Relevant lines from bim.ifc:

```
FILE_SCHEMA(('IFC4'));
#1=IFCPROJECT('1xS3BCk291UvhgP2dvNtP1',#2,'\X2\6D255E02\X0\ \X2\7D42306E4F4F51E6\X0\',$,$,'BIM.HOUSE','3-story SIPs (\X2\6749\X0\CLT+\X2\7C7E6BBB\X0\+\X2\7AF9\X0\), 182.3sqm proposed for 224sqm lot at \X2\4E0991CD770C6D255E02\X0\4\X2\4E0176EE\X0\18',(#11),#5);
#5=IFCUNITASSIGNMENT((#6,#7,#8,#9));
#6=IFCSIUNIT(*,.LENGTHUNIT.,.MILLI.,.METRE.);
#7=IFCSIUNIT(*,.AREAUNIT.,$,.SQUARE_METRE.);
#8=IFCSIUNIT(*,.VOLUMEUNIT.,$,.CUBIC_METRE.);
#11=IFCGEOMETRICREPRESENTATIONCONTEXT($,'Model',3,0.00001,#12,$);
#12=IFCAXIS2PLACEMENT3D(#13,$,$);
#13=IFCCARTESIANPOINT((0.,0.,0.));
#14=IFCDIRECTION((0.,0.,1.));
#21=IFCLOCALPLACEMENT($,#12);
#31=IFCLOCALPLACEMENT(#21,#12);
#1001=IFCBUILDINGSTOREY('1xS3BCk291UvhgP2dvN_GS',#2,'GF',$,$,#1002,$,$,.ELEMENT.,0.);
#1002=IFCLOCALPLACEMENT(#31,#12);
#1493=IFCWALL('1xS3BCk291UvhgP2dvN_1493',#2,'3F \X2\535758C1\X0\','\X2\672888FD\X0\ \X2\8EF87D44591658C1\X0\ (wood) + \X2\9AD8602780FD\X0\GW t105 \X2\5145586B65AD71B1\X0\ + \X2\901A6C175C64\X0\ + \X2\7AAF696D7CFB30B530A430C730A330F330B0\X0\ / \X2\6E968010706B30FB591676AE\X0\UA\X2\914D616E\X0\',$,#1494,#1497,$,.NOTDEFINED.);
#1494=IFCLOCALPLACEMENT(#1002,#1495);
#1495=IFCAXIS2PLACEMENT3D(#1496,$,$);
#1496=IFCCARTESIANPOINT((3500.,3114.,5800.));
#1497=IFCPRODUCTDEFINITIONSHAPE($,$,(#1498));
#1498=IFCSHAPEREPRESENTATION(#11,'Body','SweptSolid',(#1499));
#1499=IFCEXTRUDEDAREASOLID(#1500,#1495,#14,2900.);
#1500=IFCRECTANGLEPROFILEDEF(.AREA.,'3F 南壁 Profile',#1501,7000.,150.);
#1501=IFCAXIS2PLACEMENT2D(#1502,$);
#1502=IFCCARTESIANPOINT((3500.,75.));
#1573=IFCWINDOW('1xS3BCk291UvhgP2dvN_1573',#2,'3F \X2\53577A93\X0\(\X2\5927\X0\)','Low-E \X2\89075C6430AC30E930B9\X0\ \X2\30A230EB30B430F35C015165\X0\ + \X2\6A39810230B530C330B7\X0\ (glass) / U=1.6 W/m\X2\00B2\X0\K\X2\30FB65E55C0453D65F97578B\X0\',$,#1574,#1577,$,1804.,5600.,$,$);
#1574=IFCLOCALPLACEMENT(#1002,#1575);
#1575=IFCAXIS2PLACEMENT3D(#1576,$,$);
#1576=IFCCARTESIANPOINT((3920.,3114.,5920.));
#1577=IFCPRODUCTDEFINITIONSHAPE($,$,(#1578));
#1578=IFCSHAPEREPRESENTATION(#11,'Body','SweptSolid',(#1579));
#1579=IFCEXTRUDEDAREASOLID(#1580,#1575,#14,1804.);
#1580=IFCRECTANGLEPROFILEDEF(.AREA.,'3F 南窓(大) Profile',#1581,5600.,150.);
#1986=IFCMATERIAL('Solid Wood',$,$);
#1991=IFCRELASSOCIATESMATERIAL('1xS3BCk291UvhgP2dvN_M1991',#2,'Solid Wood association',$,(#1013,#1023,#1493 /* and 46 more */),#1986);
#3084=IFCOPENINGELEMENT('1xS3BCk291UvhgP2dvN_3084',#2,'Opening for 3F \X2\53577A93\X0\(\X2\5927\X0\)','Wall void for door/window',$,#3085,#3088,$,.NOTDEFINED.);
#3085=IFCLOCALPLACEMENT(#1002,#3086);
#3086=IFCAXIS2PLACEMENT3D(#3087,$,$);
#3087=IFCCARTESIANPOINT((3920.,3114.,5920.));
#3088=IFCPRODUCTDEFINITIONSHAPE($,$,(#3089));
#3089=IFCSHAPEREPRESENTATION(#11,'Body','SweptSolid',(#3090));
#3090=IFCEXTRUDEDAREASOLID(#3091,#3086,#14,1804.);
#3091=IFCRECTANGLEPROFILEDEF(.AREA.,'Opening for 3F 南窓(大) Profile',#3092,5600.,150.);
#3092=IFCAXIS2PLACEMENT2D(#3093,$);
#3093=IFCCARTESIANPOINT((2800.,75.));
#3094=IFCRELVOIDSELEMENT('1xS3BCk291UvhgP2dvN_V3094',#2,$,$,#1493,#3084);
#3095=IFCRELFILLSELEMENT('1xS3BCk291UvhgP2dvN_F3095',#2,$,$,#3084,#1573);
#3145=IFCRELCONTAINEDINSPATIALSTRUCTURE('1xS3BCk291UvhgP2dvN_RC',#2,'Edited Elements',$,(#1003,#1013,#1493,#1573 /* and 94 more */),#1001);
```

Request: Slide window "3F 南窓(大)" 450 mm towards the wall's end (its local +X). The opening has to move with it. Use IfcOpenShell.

```python
import ifcopenshell
import ifcopenshell.api.geometry
import ifcopenshell.util.placement

model = ifcopenshell.open("bim.ifc")

window = model.by_guid("1xS3BCk291UvhgP2dvN_1573")
opening = window.FillsVoids[0].RelatingOpeningElement
wall = opening.VoidsElements[0].RelatingBuildingElement

wall_matrix = ifcopenshell.util.placement.get_local_placement(wall.ObjectPlacement)
shift = wall_matrix[:3, 0] * 450.0
before = ifcopenshell.util.placement.get_local_placement(window.ObjectPlacement)[:3, 3].copy()

# The window is not placed relative to its opening, so move both.
for product in (opening, window):
    matrix = ifcopenshell.util.placement.get_local_placement(product.ObjectPlacement)
    matrix[:3, 3] += shift
    ifcopenshell.api.geometry.edit_object_placement(model, product=product, matrix=matrix, is_si=False)

after = ifcopenshell.util.placement.get_local_placement(window.ObjectPlacement)[:3, 3]
print("window moved by", (after - before).round(3) + 0.0)

model.write("bim-out.ifc")
```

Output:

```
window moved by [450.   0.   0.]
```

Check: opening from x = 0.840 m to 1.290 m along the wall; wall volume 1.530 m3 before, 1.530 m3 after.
